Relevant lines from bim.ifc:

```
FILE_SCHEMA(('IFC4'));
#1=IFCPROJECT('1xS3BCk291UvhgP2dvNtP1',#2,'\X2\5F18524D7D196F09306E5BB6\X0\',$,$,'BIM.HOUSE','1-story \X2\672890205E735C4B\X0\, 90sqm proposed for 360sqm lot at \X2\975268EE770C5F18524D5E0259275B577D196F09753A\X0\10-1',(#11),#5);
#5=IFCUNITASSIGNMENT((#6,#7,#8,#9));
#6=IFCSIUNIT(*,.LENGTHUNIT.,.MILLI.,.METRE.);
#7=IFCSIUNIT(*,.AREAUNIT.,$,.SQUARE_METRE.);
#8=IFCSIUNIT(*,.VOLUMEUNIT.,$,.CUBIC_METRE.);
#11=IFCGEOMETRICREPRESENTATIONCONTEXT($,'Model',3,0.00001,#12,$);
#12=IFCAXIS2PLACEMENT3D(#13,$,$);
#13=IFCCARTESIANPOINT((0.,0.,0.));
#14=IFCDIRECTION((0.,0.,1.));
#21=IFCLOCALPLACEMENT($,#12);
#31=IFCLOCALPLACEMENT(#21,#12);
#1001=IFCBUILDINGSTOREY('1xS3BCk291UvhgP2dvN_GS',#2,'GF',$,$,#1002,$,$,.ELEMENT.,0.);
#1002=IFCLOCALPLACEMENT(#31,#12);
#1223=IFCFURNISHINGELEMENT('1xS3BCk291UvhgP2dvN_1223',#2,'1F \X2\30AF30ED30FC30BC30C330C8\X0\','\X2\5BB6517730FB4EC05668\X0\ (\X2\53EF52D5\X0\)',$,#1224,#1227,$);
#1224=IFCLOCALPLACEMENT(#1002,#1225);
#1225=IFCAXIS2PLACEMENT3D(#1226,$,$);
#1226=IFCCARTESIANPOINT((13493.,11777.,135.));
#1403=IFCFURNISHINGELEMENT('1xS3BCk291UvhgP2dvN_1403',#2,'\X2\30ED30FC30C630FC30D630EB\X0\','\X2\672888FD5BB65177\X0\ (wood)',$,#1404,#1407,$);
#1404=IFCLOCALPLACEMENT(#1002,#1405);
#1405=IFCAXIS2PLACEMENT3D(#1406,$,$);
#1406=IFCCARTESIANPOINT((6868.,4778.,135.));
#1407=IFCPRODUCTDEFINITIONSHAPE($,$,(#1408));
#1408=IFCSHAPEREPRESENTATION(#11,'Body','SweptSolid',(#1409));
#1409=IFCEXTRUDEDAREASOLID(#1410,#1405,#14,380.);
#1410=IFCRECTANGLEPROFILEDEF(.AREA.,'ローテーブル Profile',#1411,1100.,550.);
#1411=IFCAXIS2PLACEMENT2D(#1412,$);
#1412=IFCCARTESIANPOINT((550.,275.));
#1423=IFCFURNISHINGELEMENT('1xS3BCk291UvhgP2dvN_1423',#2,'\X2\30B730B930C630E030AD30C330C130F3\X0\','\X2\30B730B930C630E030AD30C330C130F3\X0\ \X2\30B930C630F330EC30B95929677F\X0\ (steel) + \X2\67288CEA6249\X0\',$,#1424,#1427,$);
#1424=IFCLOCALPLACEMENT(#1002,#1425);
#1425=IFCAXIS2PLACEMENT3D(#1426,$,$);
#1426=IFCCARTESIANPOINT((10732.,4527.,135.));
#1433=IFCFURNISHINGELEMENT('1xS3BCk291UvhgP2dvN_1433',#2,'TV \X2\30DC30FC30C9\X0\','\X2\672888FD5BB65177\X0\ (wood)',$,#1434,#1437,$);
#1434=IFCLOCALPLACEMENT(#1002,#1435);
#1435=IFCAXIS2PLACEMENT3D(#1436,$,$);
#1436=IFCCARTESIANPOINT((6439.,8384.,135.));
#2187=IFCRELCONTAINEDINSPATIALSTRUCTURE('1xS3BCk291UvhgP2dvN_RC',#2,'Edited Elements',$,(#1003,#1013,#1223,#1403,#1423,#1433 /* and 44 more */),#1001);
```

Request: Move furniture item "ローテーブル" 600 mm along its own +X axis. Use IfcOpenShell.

```python
import ifcopenshell
import ifcopenshell.api.geometry
import ifcopenshell.util.placement

model = ifcopenshell.open("bim.ifc")

item = model.by_guid("1xS3BCk291UvhgP2dvN_1403")
matrix = ifcopenshell.util.placement.get_local_placement(item.ObjectPlacement)
matrix[:3, 3] += matrix[:3, 0] * 600.0
ifcopenshell.api.geometry.edit_object_placement(model, product=item, matrix=matrix, is_si=False)

print(ifcopenshell.util.placement.get_local_placement(item.ObjectPlacement).round(3) + 0.0)

model.write("bim_edited.ifc")
```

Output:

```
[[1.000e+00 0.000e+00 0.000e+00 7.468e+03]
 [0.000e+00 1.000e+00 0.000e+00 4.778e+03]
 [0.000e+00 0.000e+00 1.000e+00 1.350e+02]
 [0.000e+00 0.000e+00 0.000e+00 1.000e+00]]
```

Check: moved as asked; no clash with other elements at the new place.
